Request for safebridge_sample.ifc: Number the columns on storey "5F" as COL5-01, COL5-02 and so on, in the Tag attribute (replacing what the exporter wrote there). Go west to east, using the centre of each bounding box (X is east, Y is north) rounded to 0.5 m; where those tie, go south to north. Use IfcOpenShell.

First a look at what the model holds.

```python
import ifcopenshell
import ifcopenshell.util.element
import ifcopenshell.util.placement

model = ifcopenshell.open("safebridge_sample.ifc")
print(model.schema)
storey = next(s for s in model.by_type("IfcBuildingStorey") if s.Name == "5F")
columns = [e for e in ifcopenshell.util.element.get_decomposition(storey) if e.is_a("IfcColumn")]
for e in sorted(columns, key=lambda e: e.id()):
    origin = ifcopenshell.util.placement.get_local_placement(e.ObjectPlacement)[:3, 3]
    print(e.id(), e.Tag, e.Name, origin.round(2) + 0.0, sep=" | ")
```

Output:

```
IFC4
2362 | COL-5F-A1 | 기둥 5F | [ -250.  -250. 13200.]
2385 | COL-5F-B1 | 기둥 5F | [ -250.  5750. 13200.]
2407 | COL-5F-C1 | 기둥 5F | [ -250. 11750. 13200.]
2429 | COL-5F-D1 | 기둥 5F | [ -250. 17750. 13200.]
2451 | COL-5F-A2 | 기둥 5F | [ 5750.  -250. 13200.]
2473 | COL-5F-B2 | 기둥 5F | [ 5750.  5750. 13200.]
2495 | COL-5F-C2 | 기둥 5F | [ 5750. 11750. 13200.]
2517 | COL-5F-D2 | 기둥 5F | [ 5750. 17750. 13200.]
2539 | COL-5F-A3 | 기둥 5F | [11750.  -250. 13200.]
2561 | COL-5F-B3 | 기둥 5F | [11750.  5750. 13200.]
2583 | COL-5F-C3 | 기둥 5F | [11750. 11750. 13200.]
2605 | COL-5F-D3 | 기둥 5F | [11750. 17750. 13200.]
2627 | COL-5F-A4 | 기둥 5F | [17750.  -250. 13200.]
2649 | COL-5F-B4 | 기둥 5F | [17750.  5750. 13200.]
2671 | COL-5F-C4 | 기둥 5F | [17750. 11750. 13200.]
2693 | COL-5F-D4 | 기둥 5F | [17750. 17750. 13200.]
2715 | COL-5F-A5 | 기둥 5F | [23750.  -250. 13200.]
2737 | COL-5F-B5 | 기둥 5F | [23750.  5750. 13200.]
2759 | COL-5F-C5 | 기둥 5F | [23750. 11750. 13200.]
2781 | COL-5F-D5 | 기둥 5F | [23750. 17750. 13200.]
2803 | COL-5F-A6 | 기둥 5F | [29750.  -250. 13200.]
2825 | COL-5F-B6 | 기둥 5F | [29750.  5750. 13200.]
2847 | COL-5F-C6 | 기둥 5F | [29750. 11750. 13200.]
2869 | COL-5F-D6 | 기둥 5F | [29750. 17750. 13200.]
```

```python
import ifcopenshell
import ifcopenshell.geom
import ifcopenshell.util.element
import ifcopenshell.util.shape

model = ifcopenshell.open("safebridge_sample.ifc")
settings = ifcopenshell.geom.settings()
settings.set("use-world-coords", True)


def centre(element):
    shape = ifcopenshell.geom.create_shape(settings, element)
    return ifcopenshell.util.shape.get_bbox_centroid(shape.geometry)


storey = next(s for s in model.by_type("IfcBuildingStorey") if s.Name == "5F")
columns = [e for e in ifcopenshell.util.element.get_decomposition(storey) if e.is_a("IfcColumn")]

# Insertion points can sit at a corner or the storey origin, so sort by the geometry (in metres).
centres = {e: centre(e) for e in columns}
columns.sort(key=lambda e: (round(centres[e][0] / 0.5), centres[e][1]))

for i, e in enumerate(columns, start=1):
    number = f"COL5-{i:02d}"
    e.Tag = number
    print(e.id(), number)

model.write("safebridge_sample_v2.ifc")
```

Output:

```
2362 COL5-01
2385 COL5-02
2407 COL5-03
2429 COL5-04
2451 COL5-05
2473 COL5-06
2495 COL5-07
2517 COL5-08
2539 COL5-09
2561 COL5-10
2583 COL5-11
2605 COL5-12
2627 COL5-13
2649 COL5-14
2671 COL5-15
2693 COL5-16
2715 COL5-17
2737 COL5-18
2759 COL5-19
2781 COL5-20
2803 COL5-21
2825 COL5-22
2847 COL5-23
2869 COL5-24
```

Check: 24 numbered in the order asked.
